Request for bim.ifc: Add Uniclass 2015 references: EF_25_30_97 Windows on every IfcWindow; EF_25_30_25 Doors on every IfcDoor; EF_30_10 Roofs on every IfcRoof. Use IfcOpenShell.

First a look at what the model holds.

```python
import ifcopenshell

model = ifcopenshell.open("bim.ifc")
print(model.schema)
print("classifications:", [c.Name for c in model.by_type("IfcClassification")])
for ifc_class in ("IfcDoor", "IfcRoof", "IfcStair", "IfcWall", "IfcWindow"):
    print(ifc_class, len(model.by_type(ifc_class)))
```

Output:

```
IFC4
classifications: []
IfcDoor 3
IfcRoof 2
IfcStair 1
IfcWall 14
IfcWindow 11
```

```python
import ifcopenshell
import ifcopenshell.api.classification

model = ifcopenshell.open("bim.ifc")

system = ifcopenshell.api.classification.add_classification(model, classification="Uniclass 2015")

codes = {
    "IfcWindow": ("EF_25_30_97", "Windows"),
    "IfcDoor": ("EF_25_30_25", "Doors"),
    "IfcRoof": ("EF_30_10", "Roofs"),
}
for ifc_class, (code, name) in codes.items():
    products = model.by_type(ifc_class)
    ifcopenshell.api.classification.add_reference(
        model, products=products, classification=system, identification=code, name=name
    )
    print(code, len(products))

model.write("bim-out.ifc")
```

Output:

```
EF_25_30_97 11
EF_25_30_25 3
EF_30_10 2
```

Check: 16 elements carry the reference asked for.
